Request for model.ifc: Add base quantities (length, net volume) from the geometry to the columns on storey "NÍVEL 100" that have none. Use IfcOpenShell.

First a look at what the model holds.

```python
import ifcopenshell
import ifcopenshell.util.element
import ifcopenshell.util.unit

model = ifcopenshell.open("model.ifc")
print(model.schema)
for unit_type in ("LENGTHUNIT", "AREAUNIT", "VOLUMEUNIT"):
    print(unit_type, ifcopenshell.util.unit.calculate_unit_scale(model, unit_type))
storey = next(s for s in model.by_type("IfcBuildingStorey") if s.Name == "NÍVEL 100")
columns = [e for e in ifcopenshell.util.element.get_decomposition(storey) if e.is_a("IfcColumn")]
for e in sorted(columns, key=lambda e: e.id()):
    print(e.id(), e.is_a(), e.Name, list(ifcopenshell.util.element.get_psets(e, qtos_only=True)), sep=" | ")
```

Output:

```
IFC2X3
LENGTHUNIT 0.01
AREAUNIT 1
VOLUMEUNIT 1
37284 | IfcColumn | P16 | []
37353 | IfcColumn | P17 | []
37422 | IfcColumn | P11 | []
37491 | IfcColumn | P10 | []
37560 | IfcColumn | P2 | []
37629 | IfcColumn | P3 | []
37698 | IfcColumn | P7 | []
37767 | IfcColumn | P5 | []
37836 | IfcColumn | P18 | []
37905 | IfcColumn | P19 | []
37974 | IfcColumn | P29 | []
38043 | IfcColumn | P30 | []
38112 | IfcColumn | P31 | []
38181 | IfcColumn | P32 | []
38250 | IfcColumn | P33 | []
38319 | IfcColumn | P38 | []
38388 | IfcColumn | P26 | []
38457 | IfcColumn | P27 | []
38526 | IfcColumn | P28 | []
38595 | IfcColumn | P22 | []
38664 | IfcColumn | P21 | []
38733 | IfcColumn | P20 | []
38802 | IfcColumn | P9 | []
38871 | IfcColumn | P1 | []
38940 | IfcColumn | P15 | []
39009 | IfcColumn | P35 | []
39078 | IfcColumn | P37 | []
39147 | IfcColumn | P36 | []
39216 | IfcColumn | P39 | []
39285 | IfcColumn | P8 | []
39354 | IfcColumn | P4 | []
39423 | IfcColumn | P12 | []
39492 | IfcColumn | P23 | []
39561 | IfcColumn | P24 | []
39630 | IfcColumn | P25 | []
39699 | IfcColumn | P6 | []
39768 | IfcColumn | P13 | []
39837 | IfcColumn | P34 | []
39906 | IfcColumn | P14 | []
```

```python
import ifcopenshell
import ifcopenshell.api.pset
import ifcopenshell.geom
import ifcopenshell.util.element
import ifcopenshell.util.shape
import ifcopenshell.util.unit

model = ifcopenshell.open("model.ifc")
unit_scale = ifcopenshell.util.unit.calculate_unit_scale(model)
volume_scale = ifcopenshell.util.unit.calculate_unit_scale(model, "VOLUMEUNIT")
settings = ifcopenshell.geom.settings()

storey = next(s for s in model.by_type("IfcBuildingStorey") if s.Name == "NÍVEL 100")
columns = [e for e in ifcopenshell.util.element.get_decomposition(storey) if e.is_a("IfcColumn")]

for e in sorted(columns, key=lambda e: e.id()):
    if ifcopenshell.util.element.get_psets(e, qtos_only=True, should_inherit=False):
        continue
    # Geometry comes back in metres, in the element's own axes.
    shape = ifcopenshell.geom.create_shape(settings, e)
    values = {
        "Length": ifcopenshell.util.shape.get_z(shape.geometry) / unit_scale,
        "NetVolume": ifcopenshell.util.shape.get_volume(shape.geometry) / volume_scale,
    }
    qto = ifcopenshell.api.pset.add_qto(model, product=e, name="BaseQuantities")
    ifcopenshell.api.pset.edit_qto(model, qto=qto, properties=values)
    print(e.id(), {k: round(v, 3) for k, v in values.items()})

model.write("model_v2.ifc")
```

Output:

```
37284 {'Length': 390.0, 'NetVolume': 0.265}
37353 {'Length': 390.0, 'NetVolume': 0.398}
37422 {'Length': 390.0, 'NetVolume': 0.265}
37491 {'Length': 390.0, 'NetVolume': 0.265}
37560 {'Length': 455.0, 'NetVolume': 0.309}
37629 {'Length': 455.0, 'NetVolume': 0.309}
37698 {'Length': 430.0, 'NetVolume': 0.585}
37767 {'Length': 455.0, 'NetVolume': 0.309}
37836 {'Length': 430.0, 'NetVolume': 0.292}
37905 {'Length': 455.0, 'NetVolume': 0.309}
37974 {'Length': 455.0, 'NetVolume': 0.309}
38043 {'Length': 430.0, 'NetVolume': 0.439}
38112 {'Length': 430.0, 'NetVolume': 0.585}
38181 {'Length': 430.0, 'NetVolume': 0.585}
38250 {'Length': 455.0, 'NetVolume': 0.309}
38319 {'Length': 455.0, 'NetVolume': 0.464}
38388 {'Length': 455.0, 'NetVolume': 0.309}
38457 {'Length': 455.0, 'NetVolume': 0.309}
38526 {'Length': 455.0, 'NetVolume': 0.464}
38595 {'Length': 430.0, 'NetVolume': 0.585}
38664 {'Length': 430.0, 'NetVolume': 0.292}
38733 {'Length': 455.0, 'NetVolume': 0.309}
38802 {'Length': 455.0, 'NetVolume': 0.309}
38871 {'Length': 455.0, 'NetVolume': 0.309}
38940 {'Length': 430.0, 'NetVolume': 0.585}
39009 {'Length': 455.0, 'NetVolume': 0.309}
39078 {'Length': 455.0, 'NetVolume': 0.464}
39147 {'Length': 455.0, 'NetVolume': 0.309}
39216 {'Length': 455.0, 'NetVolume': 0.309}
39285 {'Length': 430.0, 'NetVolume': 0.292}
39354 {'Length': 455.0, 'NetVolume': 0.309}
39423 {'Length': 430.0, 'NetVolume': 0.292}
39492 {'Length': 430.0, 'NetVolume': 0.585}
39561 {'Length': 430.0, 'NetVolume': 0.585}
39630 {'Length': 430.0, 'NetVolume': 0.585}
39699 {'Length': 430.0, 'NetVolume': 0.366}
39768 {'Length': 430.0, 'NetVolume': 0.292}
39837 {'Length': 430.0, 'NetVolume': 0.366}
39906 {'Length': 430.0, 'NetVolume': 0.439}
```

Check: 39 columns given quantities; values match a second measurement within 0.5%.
